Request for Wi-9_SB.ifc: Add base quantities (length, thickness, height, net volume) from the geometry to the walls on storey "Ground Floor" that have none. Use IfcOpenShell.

First a look at what the model holds.

```python
import ifcopenshell
import ifcopenshell.util.element
import ifcopenshell.util.unit

model = ifcopenshell.open("Wi-9_SB.ifc")
print(model.schema)
for unit_type in ("LENGTHUNIT", "AREAUNIT", "VOLUMEUNIT"):
    print(unit_type, ifcopenshell.util.unit.calculate_unit_scale(model, unit_type))
storey = next(s for s in model.by_type("IfcBuildingStorey") if s.Name == "Ground Floor")
walls = [e for e in ifcopenshell.util.element.get_decomposition(storey) if e.is_a("IfcWall")]
for e in sorted(walls, key=lambda e: e.id()):
    print(e.id(), e.is_a(), e.Name, list(ifcopenshell.util.element.get_psets(e, qtos_only=True)), sep=" | ")
```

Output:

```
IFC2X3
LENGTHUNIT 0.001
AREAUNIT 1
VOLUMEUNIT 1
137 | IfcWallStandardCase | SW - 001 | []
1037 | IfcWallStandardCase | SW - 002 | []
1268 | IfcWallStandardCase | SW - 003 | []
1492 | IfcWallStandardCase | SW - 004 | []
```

```python
import ifcopenshell
import ifcopenshell.api.pset
import ifcopenshell.geom
import ifcopenshell.util.element
import ifcopenshell.util.shape
import ifcopenshell.util.unit

model = ifcopenshell.open("Wi-9_SB.ifc")
unit_scale = ifcopenshell.util.unit.calculate_unit_scale(model)
volume_scale = ifcopenshell.util.unit.calculate_unit_scale(model, "VOLUMEUNIT")
settings = ifcopenshell.geom.settings()

storey = next(s for s in model.by_type("IfcBuildingStorey") if s.Name == "Ground Floor")
walls = [e for e in ifcopenshell.util.element.get_decomposition(storey) if e.is_a("IfcWall")]

for e in sorted(walls, key=lambda e: e.id()):
    if ifcopenshell.util.element.get_psets(e, qtos_only=True, should_inherit=False):
        continue
    # Geometry comes back in metres, in the element's own axes.
    shape = ifcopenshell.geom.create_shape(settings, e)
    values = {
        "Length": ifcopenshell.util.shape.get_x(shape.geometry) / unit_scale,
        "Width": ifcopenshell.util.shape.get_y(shape.geometry) / unit_scale,
        "Height": ifcopenshell.util.shape.get_z(shape.geometry) / unit_scale,
        "NetVolume": ifcopenshell.util.shape.get_volume(shape.geometry) / volume_scale,
    }
    qto = ifcopenshell.api.pset.add_qto(model, product=e, name="BaseQuantities")
    ifcopenshell.api.pset.edit_qto(model, qto=qto, properties=values)
    print(e.id(), {k: round(v, 3) for k, v in values.items()})

model.write("Wi-9_SB-out.ifc")
```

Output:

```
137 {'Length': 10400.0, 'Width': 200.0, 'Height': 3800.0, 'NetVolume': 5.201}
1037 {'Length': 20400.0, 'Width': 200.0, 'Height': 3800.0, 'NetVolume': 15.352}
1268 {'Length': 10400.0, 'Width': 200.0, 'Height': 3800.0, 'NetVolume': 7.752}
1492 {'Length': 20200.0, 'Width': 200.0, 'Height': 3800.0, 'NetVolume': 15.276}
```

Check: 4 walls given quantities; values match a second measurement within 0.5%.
